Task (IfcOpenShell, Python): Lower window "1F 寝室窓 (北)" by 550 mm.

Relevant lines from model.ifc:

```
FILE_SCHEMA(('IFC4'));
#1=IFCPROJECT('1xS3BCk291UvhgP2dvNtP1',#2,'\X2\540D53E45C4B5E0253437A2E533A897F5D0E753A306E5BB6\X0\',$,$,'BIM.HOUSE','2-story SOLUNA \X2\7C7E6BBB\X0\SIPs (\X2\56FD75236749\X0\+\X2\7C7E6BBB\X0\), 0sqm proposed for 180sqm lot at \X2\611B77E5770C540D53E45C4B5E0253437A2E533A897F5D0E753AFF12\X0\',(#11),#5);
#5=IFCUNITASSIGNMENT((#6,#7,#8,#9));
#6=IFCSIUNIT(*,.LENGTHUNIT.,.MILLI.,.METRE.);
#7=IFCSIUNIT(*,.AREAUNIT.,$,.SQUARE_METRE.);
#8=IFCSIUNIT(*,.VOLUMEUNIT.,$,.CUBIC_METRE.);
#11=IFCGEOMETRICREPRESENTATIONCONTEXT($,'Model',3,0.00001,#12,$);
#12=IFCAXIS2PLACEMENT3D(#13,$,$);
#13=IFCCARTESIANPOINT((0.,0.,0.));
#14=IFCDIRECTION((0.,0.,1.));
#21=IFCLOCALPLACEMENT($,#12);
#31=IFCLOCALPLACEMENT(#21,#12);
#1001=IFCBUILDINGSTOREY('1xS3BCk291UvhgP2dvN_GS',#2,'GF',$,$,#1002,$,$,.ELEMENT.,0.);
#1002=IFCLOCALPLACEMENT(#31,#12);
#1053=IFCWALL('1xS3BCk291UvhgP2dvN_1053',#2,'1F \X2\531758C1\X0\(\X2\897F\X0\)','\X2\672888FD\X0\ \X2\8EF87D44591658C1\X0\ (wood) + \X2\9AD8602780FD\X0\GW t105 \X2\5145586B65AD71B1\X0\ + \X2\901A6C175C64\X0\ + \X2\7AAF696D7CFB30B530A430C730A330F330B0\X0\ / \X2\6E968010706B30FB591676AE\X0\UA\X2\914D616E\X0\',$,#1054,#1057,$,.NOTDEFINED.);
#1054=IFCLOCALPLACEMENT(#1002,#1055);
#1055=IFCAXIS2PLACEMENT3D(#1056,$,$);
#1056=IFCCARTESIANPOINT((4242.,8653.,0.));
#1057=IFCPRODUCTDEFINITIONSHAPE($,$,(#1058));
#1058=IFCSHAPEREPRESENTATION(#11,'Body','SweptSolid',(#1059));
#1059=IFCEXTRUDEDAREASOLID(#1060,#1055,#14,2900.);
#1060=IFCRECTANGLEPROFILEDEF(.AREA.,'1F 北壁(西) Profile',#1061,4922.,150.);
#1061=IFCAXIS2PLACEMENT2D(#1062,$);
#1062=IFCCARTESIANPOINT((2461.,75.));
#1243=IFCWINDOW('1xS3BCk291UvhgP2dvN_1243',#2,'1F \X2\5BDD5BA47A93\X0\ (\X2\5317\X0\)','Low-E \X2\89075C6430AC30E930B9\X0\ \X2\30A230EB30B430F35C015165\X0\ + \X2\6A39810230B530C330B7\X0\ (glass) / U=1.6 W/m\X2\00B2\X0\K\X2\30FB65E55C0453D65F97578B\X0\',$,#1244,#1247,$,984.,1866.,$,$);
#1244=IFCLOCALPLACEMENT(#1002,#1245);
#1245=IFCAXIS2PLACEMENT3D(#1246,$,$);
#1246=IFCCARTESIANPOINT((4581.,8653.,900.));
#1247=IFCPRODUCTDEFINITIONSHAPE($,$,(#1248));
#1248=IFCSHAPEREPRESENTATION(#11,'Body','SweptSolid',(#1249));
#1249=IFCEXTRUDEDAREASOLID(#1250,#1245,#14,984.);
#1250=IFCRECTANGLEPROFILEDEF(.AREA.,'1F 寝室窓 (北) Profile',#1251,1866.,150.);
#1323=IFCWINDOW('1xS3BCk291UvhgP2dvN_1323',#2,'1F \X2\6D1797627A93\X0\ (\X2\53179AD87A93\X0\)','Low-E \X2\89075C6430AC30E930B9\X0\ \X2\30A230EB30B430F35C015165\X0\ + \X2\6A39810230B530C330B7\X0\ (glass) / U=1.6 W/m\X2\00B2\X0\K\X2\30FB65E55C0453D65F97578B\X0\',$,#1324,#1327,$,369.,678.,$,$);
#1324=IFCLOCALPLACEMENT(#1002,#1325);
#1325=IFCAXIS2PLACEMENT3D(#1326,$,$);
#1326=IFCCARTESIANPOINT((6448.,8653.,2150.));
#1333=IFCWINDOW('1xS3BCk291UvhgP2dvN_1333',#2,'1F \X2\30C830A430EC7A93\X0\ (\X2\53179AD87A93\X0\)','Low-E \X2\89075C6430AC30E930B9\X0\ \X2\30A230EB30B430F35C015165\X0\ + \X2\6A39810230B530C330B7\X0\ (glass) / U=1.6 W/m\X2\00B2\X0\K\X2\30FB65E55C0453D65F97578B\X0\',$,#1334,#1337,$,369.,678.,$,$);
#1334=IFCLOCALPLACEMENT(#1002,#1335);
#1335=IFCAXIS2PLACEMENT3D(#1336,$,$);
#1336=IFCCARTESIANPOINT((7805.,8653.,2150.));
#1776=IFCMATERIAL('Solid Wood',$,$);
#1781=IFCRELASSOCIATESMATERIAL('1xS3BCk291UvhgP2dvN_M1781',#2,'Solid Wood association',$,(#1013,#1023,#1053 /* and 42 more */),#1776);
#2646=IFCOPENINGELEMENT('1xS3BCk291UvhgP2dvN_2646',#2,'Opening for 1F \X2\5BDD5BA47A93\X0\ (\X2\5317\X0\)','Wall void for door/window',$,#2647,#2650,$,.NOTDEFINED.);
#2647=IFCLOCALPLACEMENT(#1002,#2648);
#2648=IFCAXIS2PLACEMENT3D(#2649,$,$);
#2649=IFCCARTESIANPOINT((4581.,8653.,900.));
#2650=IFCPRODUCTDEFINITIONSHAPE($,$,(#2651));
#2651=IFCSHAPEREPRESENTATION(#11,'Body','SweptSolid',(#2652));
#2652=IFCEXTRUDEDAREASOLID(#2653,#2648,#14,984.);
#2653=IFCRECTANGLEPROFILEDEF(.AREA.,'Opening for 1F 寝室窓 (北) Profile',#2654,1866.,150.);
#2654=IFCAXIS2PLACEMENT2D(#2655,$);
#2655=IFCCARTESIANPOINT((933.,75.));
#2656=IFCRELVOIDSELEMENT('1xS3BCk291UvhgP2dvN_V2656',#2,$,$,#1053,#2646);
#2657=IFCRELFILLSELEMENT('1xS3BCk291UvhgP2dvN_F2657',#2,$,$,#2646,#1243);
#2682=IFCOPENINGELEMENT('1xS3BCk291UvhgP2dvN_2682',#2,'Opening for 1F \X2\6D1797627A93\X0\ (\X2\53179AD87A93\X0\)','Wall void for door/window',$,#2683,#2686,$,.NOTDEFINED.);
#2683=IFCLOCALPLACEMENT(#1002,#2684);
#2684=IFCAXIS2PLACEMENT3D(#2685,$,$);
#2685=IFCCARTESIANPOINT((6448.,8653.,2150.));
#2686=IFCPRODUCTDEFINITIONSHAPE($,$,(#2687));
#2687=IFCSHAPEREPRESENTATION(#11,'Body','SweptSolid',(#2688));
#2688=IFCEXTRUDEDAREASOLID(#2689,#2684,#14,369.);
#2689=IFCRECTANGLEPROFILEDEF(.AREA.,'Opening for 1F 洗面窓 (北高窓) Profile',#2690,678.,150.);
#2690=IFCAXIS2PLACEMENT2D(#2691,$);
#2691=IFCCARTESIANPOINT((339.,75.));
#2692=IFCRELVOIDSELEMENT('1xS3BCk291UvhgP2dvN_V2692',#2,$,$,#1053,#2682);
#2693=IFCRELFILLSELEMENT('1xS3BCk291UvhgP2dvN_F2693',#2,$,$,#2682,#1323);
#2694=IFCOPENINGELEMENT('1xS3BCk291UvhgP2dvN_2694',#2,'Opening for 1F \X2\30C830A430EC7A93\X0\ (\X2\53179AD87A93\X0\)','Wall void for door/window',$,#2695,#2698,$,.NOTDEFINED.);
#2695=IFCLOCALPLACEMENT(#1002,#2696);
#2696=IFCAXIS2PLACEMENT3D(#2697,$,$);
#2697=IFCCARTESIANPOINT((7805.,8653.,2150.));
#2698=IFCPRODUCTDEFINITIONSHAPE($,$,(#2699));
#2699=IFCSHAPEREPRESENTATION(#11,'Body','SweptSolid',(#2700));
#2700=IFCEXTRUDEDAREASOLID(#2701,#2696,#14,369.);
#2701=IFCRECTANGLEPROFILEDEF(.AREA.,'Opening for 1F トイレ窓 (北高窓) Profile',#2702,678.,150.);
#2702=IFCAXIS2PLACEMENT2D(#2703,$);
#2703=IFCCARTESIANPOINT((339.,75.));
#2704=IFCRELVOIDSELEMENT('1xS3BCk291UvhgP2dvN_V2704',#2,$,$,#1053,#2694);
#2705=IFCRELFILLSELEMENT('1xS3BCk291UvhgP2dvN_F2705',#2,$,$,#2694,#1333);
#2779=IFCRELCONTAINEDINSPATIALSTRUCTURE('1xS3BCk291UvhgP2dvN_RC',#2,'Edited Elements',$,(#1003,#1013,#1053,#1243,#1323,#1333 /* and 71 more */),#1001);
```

```python
import numpy as np
import ifcopenshell
import ifcopenshell.api.geometry
import ifcopenshell.util.placement
import ifcopenshell.util.unit

model = ifcopenshell.open("model.ifc")
unit_scale = ifcopenshell.util.unit.calculate_unit_scale(model)

window = model.by_id(1243)
opening = window.FillsVoids[0].RelatingOpeningElement
dz = -0.55 / unit_scale

shift = np.array([0.0, 0.0, dz])
# The window is not placed relative to its opening, so move both.
for product in (opening, window):
    matrix = ifcopenshell.util.placement.get_local_placement(product.ObjectPlacement)
    matrix[:3, 3] += shift
    ifcopenshell.api.geometry.edit_object_placement(model, product=product, matrix=matrix, is_si=False)

print(f"moved by {dz * unit_scale:+.3f} m")

model.write("model_v2.ifc")
```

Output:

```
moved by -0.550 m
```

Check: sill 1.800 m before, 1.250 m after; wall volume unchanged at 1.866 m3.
